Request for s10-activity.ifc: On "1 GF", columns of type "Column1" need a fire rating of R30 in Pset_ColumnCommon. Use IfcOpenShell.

First a look at what the model holds.

```python
import ifcopenshell
import ifcopenshell.util.element

model = ifcopenshell.open("s10-activity.ifc")
print(model.schema)
storey = next(s for s in model.by_type("IfcBuildingStorey") if s.Name == "1 GF")
columns = [e for e in ifcopenshell.util.element.get_decomposition(storey) if e.is_a("IfcColumn")]
seen = {}
for e in columns:
    element_type = ifcopenshell.util.element.get_type(e)
    key = (element_type.Name if element_type != e and element_type else None, ifcopenshell.util.element.get_pset(e, "Pset_ColumnCommon", "FireRating"))
    seen[key] = seen.get(key, 0) + 1
for (name, value), count in sorted(seen.items(), key=str):
    print(count, "x", name, "|", value)
```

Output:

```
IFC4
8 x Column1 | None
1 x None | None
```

```python
import ifcopenshell
import ifcopenshell.api.pset
import ifcopenshell.util.element

model = ifcopenshell.open("s10-activity.ifc")

storey = next(s for s in model.by_type("IfcBuildingStorey") if s.Name == "1 GF")
columns = [e for e in ifcopenshell.util.element.get_decomposition(storey) if e.is_a("IfcColumn")]

count = 0
for e in columns:
    element_type = ifcopenshell.util.element.get_type(e)
    if element_type in (None, e) or element_type.Name != "Column1":
        continue
    # add_pset returns the element's existing set when there is one.
    pset = ifcopenshell.api.pset.add_pset(model, product=e, name="Pset_ColumnCommon")
    ifcopenshell.api.pset.edit_pset(model, pset=pset, properties={"FireRating": "R30"})
    count += 1

print(count, "columns updated")

model.write("s10-activity_v2.ifc")
```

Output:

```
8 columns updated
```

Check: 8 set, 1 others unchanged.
